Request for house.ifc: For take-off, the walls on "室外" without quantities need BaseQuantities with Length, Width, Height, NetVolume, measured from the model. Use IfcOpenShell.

First a look at what the model holds.

```python
import ifcopenshell
import ifcopenshell.util.element
import ifcopenshell.util.unit

model = ifcopenshell.open("house.ifc")
print(model.schema)
for unit_type in ("LENGTHUNIT", "AREAUNIT", "VOLUMEUNIT"):
    print(unit_type, ifcopenshell.util.unit.calculate_unit_scale(model, unit_type))
storey = next(s for s in model.by_type("IfcBuildingStorey") if s.Name == "室外")
walls = [e for e in ifcopenshell.util.element.get_decomposition(storey) if e.is_a("IfcWall")]
for e in sorted(walls, key=lambda e: e.id()):
    print(e.id(), e.is_a(), e.Name, list(ifcopenshell.util.element.get_psets(e, qtos_only=True)), sep=" | ")
```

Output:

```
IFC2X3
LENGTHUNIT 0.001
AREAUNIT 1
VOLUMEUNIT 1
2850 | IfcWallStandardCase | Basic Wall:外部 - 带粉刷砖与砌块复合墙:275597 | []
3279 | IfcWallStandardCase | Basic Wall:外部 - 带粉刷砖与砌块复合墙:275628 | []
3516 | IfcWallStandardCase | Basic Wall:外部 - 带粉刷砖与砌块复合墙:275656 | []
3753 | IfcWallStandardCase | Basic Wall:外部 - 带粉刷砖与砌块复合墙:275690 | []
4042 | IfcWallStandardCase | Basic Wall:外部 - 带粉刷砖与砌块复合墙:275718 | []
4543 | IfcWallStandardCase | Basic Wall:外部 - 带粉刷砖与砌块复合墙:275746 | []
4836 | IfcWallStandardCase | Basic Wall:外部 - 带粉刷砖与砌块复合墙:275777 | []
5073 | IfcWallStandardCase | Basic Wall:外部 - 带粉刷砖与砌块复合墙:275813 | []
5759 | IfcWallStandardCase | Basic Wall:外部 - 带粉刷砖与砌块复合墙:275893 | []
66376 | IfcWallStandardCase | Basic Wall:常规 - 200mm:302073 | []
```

```python
import ifcopenshell
import ifcopenshell.api.pset
import ifcopenshell.geom
import ifcopenshell.util.element
import ifcopenshell.util.shape
import ifcopenshell.util.unit

model = ifcopenshell.open("house.ifc")
unit_scale = ifcopenshell.util.unit.calculate_unit_scale(model)
volume_scale = ifcopenshell.util.unit.calculate_unit_scale(model, "VOLUMEUNIT")
settings = ifcopenshell.geom.settings()

storey = next(s for s in model.by_type("IfcBuildingStorey") if s.Name == "室外")
walls = [e for e in ifcopenshell.util.element.get_decomposition(storey) if e.is_a("IfcWall")]

for e in sorted(walls, key=lambda e: e.id()):
    if ifcopenshell.util.element.get_psets(e, qtos_only=True, should_inherit=False):
        continue
    # Geometry comes back in metres, in the element's own axes.
    shape = ifcopenshell.geom.create_shape(settings, e)
    values = {
        "Length": ifcopenshell.util.shape.get_x(shape.geometry) / unit_scale,
        "Width": ifcopenshell.util.shape.get_y(shape.geometry) / unit_scale,
        "Height": ifcopenshell.util.shape.get_z(shape.geometry) / unit_scale,
        "NetVolume": ifcopenshell.util.shape.get_volume(shape.geometry) / volume_scale,
    }
    qto = ifcopenshell.api.pset.add_qto(model, product=e, name="BaseQuantities")
    ifcopenshell.api.pset.edit_qto(model, qto=qto, properties=values)
    print(e.id(), {k: round(v, 3) for k, v in values.items()})

model.write("house_updated.ifc")
```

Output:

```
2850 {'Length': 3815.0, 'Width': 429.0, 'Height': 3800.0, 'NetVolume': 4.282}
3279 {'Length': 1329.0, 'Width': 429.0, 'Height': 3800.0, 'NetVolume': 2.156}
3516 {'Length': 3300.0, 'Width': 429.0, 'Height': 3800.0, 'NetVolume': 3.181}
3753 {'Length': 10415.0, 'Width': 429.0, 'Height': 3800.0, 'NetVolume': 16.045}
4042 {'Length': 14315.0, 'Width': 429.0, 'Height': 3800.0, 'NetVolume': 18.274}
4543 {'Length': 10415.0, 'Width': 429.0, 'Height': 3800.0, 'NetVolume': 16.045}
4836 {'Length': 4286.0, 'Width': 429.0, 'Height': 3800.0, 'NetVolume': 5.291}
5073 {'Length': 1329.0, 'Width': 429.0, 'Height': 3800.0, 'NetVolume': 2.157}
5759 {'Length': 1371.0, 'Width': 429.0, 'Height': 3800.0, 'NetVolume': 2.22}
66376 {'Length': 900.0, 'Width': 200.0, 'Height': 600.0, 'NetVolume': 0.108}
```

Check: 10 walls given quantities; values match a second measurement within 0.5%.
